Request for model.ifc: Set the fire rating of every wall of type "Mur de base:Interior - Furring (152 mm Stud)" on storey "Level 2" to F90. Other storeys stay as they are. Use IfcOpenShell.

First a look at what the model holds.

```python
import ifcopenshell
import ifcopenshell.util.element

model = ifcopenshell.open("model.ifc")
print(model.schema)
storey = next(s for s in model.by_type("IfcBuildingStorey") if s.Name == "Level 2")
walls = [e for e in ifcopenshell.util.element.get_decomposition(storey) if e.is_a("IfcWall")]
seen = {}
for e in walls:
    element_type = ifcopenshell.util.element.get_type(e)
    key = (element_type.Name if element_type != e and element_type else None, ifcopenshell.util.element.get_pset(e, "Pset_WallCommon", "FireRating"))
    seen[key] = seen.get(key, 0) + 1
for (name, value), count in sorted(seen.items(), key=str):
    print(count, "x", name, "|", value)
```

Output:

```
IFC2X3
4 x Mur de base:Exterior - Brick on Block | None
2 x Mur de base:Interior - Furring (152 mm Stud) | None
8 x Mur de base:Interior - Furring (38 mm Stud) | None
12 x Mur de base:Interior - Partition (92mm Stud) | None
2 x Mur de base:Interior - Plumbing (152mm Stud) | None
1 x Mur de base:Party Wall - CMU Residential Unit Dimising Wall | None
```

```python
import ifcopenshell
import ifcopenshell.api.pset
import ifcopenshell.util.element

model = ifcopenshell.open("model.ifc")

storey = next(s for s in model.by_type("IfcBuildingStorey") if s.Name == "Level 2")
walls = [e for e in ifcopenshell.util.element.get_decomposition(storey) if e.is_a("IfcWall")]

count = 0
for e in walls:
    element_type = ifcopenshell.util.element.get_type(e)
    if element_type in (None, e) or element_type.Name != "Mur de base:Interior - Furring (152 mm Stud)":
        continue
    # add_pset returns the element's existing set when there is one.
    pset = ifcopenshell.api.pset.add_pset(model, product=e, name="Pset_WallCommon")
    ifcopenshell.api.pset.edit_pset(model, pset=pset, properties={"FireRating": "F90"})
    count += 1

print(count, "walls updated")

model.write("model_v2.ifc")
```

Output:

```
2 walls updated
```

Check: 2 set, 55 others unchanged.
